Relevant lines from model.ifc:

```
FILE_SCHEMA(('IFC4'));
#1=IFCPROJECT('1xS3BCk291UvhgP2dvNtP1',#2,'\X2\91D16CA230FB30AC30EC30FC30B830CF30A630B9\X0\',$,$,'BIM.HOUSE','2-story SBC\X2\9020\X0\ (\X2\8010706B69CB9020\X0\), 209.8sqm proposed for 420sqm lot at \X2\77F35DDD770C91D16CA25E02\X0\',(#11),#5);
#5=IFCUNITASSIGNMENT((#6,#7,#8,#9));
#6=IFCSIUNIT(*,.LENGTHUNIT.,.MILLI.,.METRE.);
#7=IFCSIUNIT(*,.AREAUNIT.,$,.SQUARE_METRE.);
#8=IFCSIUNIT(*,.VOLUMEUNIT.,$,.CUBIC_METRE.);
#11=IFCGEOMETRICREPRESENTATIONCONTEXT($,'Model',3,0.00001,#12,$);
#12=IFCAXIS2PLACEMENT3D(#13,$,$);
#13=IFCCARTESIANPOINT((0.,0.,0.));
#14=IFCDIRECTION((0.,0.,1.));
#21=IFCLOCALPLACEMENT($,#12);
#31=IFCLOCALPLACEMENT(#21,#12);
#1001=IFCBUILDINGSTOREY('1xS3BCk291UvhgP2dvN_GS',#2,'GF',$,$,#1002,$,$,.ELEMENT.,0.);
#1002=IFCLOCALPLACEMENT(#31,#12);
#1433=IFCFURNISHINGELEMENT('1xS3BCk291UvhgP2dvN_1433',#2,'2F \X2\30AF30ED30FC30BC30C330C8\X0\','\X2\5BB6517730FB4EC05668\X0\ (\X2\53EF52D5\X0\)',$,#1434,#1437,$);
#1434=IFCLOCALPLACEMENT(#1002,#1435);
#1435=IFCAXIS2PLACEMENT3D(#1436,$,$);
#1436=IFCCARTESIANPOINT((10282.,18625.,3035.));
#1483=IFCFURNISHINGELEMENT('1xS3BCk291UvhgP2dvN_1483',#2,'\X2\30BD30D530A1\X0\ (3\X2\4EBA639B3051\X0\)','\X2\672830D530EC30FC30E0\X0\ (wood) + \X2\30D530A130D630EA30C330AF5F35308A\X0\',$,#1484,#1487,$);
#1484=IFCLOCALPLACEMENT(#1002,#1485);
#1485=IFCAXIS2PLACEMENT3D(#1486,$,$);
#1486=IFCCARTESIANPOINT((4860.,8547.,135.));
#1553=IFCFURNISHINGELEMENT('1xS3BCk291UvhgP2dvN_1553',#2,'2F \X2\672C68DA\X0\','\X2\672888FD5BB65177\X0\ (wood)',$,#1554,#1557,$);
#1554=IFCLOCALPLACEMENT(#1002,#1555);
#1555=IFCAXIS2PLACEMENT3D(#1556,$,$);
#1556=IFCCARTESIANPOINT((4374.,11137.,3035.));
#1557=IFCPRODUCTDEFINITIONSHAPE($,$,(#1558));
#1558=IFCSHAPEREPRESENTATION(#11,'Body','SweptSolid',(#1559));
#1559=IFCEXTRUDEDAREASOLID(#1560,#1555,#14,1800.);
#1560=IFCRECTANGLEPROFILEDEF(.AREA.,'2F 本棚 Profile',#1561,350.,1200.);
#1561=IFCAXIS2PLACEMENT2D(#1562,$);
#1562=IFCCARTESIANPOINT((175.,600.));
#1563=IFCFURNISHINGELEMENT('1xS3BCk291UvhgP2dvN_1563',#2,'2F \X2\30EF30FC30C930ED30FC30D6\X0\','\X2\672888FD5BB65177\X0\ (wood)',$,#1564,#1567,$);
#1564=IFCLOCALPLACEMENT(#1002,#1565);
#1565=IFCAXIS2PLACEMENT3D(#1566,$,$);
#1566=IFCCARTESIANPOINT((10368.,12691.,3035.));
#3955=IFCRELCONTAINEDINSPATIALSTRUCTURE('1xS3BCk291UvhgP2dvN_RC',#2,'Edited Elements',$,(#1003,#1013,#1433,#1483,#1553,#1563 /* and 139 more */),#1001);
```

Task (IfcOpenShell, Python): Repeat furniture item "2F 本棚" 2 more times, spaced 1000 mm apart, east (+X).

```python
import numpy as np
import ifcopenshell
import ifcopenshell.api.geometry
import ifcopenshell.api.root
import ifcopenshell.util.element
import ifcopenshell.util.placement
import ifcopenshell.util.unit

model = ifcopenshell.open("model.ifc")
unit_scale = ifcopenshell.util.unit.calculate_unit_scale(model)


def reuse_history(source, copy):
    """copy_class also copies each property set's owner history, people and application; keep the originals."""
    for rel in copy.IsDefinedBy:
        if rel.is_a("IfcRelDefinesByProperties") and (history := rel.RelatingPropertyDefinition.OwnerHistory):
            rel.RelatingPropertyDefinition.OwnerHistory = source.OwnerHistory
            ifcopenshell.util.element.remove_deep2(model, history)


source = model.by_id(1553)
base = ifcopenshell.util.placement.get_local_placement(source.ObjectPlacement)
step = np.array([1.0, 0.0, 0.0]) * 1 / unit_scale

for i in range(1, 3):
    copy = ifcopenshell.api.root.copy_class(model, product=source)
    copy.Representation = ifcopenshell.util.element.copy_deep(
        model, source.Representation, exclude=["IfcGeometricRepresentationContext", "IfcRepresentationMap"]
    )
    reuse_history(source, copy)
    matrix = base.copy()
    matrix[:3, 3] += i * step
    print("added at", matrix[:3, 3].round(3) + 0.0)
    ifcopenshell.api.geometry.edit_object_placement(model, product=copy, matrix=matrix, is_si=False)

model.write("model-out.ifc")
```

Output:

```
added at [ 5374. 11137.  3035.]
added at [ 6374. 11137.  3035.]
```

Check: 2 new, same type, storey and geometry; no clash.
